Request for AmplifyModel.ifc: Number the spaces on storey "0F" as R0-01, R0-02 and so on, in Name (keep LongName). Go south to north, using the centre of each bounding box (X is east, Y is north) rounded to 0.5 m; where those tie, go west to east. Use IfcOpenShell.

First a look at what the model holds.

```python
import ifcopenshell
import ifcopenshell.util.element
import ifcopenshell.util.placement

model = ifcopenshell.open("AmplifyModel.ifc")
print(model.schema)
storey = next(s for s in model.by_type("IfcBuildingStorey") if s.Name == "0F")
spaces = [e for e in ifcopenshell.util.element.get_decomposition(storey) if e.is_a("IfcSpace")]
for e in sorted(spaces, key=lambda e: e.id()):
    origin = ifcopenshell.util.placement.get_local_placement(e.ObjectPlacement)[:3, 3]
    print(e.id(), e.Name, e.LongName, origin.round(2) + 0.0, sep=" | ")
```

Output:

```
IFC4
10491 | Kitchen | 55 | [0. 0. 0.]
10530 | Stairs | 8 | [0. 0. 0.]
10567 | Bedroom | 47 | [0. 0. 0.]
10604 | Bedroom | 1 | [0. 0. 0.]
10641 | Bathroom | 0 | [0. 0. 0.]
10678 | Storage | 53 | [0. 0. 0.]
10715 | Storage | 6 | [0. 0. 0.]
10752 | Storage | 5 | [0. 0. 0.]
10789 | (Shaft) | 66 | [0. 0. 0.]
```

```python
import ifcopenshell
import ifcopenshell.geom
import ifcopenshell.util.element
import ifcopenshell.util.shape

model = ifcopenshell.open("AmplifyModel.ifc")
settings = ifcopenshell.geom.settings()
settings.set("use-world-coords", True)


def centre(element):
    shape = ifcopenshell.geom.create_shape(settings, element)
    return ifcopenshell.util.shape.get_bbox_centroid(shape.geometry)


storey = next(s for s in model.by_type("IfcBuildingStorey") if s.Name == "0F")
spaces = [e for e in ifcopenshell.util.element.get_decomposition(storey) if e.is_a("IfcSpace")]

# Insertion points can sit at a corner or the storey origin, so sort by the geometry (in metres).
centres = {e: centre(e) for e in spaces}
spaces.sort(key=lambda e: (round(centres[e][1] / 0.5), centres[e][0]))

for i, e in enumerate(spaces, start=1):
    number = f"R0-{i:02d}"
    e.Name = number
    print(e.id(), number)

model.write("AmplifyModel_edited.ifc")
```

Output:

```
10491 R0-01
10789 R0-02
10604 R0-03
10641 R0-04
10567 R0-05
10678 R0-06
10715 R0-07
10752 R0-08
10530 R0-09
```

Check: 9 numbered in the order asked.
